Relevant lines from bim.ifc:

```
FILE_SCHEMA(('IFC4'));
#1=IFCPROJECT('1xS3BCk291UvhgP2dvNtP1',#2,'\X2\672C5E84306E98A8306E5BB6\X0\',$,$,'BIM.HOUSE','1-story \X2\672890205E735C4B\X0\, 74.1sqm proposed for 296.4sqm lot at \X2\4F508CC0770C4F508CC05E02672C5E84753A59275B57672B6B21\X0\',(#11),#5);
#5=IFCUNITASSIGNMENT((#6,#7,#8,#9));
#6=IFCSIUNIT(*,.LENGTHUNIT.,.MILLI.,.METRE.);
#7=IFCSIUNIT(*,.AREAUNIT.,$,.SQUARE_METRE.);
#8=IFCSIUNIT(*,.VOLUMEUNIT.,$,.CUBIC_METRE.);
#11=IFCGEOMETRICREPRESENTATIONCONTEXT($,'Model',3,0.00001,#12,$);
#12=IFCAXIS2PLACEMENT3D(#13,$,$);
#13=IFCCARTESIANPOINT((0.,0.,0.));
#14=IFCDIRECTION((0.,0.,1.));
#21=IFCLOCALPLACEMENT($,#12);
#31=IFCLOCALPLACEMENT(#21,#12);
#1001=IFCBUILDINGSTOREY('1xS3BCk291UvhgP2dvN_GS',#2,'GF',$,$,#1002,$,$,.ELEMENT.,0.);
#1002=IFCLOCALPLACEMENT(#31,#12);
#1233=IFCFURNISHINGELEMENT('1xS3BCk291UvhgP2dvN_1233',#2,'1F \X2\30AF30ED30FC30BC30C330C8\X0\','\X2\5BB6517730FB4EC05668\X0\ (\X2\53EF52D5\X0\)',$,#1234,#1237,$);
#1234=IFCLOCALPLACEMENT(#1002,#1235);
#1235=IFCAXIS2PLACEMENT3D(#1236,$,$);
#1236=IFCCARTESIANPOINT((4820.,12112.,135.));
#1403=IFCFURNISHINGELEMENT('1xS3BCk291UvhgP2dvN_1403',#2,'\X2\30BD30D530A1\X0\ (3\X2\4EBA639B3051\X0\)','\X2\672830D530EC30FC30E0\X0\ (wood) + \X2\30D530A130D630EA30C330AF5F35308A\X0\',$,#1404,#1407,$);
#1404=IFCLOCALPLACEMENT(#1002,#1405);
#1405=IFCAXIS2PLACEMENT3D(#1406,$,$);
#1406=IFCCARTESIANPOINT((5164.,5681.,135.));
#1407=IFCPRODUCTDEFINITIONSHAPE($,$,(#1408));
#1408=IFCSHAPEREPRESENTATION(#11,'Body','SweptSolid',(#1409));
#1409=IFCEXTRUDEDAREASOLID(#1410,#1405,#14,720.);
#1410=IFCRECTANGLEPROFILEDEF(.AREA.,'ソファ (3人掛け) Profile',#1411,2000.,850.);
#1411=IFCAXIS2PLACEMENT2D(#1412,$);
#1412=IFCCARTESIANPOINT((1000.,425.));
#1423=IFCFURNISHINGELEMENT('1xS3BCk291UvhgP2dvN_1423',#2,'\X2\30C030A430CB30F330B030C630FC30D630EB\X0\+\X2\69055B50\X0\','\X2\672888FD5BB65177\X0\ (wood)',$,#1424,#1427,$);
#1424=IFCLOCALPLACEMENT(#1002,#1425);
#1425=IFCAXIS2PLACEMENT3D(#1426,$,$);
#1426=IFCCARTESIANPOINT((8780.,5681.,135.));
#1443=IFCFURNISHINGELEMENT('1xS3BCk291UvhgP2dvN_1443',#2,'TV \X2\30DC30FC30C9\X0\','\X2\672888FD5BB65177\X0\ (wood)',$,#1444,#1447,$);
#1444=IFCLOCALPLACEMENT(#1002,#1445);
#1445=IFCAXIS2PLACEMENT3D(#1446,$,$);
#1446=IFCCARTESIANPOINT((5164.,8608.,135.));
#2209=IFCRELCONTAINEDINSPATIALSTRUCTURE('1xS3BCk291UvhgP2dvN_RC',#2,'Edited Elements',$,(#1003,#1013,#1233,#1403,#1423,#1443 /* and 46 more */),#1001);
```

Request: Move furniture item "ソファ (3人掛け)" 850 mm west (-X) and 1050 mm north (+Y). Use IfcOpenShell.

```python
import ifcopenshell
import ifcopenshell.api.geometry
import ifcopenshell.util.placement

model = ifcopenshell.open("bim.ifc")

item = model.by_guid("1xS3BCk291UvhgP2dvN_1403")
matrix = ifcopenshell.util.placement.get_local_placement(item.ObjectPlacement)
matrix[0, 3] -= 850.0
matrix[1, 3] += 1050.0
ifcopenshell.api.geometry.edit_object_placement(model, product=item, matrix=matrix, is_si=False)

print(ifcopenshell.util.placement.get_local_placement(item.ObjectPlacement).round(3) + 0.0)

model.write("bim_v2.ifc")
```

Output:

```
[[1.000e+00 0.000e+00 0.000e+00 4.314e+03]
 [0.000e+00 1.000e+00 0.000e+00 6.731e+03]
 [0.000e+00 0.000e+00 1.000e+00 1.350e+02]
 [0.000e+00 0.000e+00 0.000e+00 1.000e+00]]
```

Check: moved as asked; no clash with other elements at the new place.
